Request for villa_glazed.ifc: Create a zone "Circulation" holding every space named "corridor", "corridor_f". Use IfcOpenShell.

First a look at what the model holds.

```python
import ifcopenshell

model = ifcopenshell.open("villa_glazed.ifc")
print(model.schema)
seen = {}
for space in model.by_type("IfcSpace"):
    seen[space.LongName] = seen.get(space.LongName, 0) + 1
for name, count in sorted(seen.items(), key=str):
    print(count, "x", name)
print("zones:", [z.Name for z in model.by_type("IfcZone")][:20])
```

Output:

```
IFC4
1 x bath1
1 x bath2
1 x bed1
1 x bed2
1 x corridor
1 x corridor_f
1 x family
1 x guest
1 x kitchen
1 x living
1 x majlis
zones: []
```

```python
import ifcopenshell
import ifcopenshell.api.group
import ifcopenshell.api.root

model = ifcopenshell.open("villa_glazed.ifc")

names = {"corridor", "corridor_f"}
spaces = [s for s in model.by_type("IfcSpace") if s.LongName in names]

zone = ifcopenshell.api.root.create_entity(model, ifc_class="IfcZone", name="Circulation")
ifcopenshell.api.group.assign_group(model, products=spaces, group=zone)
print(len(spaces), "spaces in", zone.Name)

model.write("villa_glazed-out.ifc")
```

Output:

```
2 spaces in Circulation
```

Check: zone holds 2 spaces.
